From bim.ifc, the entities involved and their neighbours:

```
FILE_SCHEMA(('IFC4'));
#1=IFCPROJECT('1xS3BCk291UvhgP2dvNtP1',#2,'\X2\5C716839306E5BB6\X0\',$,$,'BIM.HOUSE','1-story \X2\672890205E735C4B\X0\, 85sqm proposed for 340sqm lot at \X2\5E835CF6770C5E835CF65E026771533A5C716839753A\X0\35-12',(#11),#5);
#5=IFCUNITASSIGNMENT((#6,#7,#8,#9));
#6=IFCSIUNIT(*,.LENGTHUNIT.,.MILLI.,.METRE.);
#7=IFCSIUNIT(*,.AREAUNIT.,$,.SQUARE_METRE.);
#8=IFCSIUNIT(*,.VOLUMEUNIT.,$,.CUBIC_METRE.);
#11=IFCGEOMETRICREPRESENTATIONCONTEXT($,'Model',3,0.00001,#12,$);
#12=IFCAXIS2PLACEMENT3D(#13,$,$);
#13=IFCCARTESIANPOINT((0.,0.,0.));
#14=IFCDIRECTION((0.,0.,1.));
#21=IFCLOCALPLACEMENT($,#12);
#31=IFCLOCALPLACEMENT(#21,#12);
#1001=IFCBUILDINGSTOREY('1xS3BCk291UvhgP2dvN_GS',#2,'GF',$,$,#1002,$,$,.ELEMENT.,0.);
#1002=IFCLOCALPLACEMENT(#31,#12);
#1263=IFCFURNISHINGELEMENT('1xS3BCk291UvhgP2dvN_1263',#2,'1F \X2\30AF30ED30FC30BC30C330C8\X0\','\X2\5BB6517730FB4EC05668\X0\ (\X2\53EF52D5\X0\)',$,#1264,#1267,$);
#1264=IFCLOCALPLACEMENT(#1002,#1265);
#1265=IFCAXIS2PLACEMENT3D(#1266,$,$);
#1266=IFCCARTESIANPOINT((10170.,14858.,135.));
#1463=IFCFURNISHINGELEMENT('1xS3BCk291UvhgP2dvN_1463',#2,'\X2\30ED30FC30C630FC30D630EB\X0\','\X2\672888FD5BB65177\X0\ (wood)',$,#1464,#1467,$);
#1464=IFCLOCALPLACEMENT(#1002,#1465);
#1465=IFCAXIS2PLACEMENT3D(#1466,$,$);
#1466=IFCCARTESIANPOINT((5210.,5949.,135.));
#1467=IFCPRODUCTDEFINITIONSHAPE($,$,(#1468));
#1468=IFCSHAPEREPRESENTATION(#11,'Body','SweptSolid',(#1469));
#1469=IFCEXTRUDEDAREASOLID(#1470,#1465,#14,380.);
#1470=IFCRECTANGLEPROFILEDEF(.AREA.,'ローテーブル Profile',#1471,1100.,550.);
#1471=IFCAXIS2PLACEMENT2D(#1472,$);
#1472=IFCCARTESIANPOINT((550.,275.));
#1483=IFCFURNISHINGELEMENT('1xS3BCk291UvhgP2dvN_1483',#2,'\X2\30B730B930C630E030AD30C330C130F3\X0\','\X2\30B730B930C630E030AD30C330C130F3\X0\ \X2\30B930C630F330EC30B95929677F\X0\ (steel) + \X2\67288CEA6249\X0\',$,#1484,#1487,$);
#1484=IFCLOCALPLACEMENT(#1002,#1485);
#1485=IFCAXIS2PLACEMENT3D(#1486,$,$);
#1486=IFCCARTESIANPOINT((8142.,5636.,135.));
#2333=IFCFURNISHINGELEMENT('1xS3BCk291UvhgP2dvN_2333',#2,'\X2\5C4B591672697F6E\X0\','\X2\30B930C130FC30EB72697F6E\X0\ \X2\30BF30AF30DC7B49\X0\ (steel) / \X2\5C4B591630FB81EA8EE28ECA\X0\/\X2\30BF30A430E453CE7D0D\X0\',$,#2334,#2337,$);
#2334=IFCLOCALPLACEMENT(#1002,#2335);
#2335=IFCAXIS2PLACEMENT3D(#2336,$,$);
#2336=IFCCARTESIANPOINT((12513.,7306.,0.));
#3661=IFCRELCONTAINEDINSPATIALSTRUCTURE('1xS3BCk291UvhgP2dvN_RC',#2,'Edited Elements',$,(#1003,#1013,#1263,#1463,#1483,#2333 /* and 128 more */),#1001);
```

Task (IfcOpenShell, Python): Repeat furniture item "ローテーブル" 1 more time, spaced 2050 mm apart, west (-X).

```python
import numpy as np
import ifcopenshell
import ifcopenshell.api.geometry
import ifcopenshell.api.root
import ifcopenshell.util.element
import ifcopenshell.util.placement

model = ifcopenshell.open("bim.ifc")


def reuse_history(source, copy):
    """copy_class also copies each property set's owner history, people and application; keep the originals."""
    for rel in copy.IsDefinedBy:
        if rel.is_a("IfcRelDefinesByProperties") and (history := rel.RelatingPropertyDefinition.OwnerHistory):
            rel.RelatingPropertyDefinition.OwnerHistory = source.OwnerHistory
            ifcopenshell.util.element.remove_deep2(model, history)


source = model.by_guid("1xS3BCk291UvhgP2dvN_1463")
base = ifcopenshell.util.placement.get_local_placement(source.ObjectPlacement)
step = np.array([-1.0, 0.0, 0.0]) * 2050.0

for i in range(1, 2):
    copy = ifcopenshell.api.root.copy_class(model, product=source)
    copy.Representation = ifcopenshell.util.element.copy_deep(
        model, source.Representation, exclude=["IfcGeometricRepresentationContext", "IfcRepresentationMap"]
    )
    reuse_history(source, copy)
    matrix = base.copy()
    matrix[:3, 3] += i * step
    print("added at", matrix[:3, 3].round(3) + 0.0)
    ifcopenshell.api.geometry.edit_object_placement(model, product=copy, matrix=matrix, is_si=False)

model.write("bim_updated.ifc")
```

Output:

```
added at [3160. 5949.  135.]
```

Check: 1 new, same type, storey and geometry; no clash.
